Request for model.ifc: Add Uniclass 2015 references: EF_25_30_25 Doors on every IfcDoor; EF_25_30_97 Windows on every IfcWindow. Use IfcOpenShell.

First a look at what the model holds.

```python
import ifcopenshell

model = ifcopenshell.open("model.ifc")
print(model.schema)
print("classifications:", [c.Name for c in model.by_type("IfcClassification")])
for ifc_class in ("IfcDoor", "IfcRoof", "IfcStair", "IfcWall", "IfcWindow"):
    print(ifc_class, len(model.by_type(ifc_class)))
```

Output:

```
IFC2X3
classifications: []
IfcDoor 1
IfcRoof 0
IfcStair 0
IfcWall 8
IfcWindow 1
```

```python
import ifcopenshell
import ifcopenshell.api.classification

model = ifcopenshell.open("model.ifc")

# IFC2X3 requires Source and Edition and has no link from the project to the system.
system = model.create_entity("IfcClassification", Source="NBS", Edition="2015", Name="Uniclass 2015")

codes = {
    "IfcDoor": ("EF_25_30_25", "Doors"),
    "IfcWindow": ("EF_25_30_97", "Windows"),
}
for ifc_class, (code, name) in codes.items():
    products = model.by_type(ifc_class)
    ifcopenshell.api.classification.add_reference(
        model, products=products, classification=system, identification=code, name=name
    )
    print(code, len(products))

model.write("model-out.ifc")
```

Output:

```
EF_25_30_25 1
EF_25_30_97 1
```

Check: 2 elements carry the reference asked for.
